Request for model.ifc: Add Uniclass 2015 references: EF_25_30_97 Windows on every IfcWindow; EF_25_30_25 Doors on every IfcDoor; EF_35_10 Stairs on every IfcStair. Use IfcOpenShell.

First a look at what the model holds.

```python
import ifcopenshell

model = ifcopenshell.open("model.ifc")
print(model.schema)
print("classifications:", [c.Name for c in model.by_type("IfcClassification")])
for ifc_class in ("IfcDoor", "IfcRoof", "IfcStair", "IfcWall", "IfcWindow"):
    print(ifc_class, len(model.by_type(ifc_class)))
```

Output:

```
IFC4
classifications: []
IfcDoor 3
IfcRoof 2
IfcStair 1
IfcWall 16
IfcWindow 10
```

```python
import ifcopenshell
import ifcopenshell.api.classification

model = ifcopenshell.open("model.ifc")

system = ifcopenshell.api.classification.add_classification(model, classification="Uniclass 2015")

codes = {
    "IfcWindow": ("EF_25_30_97", "Windows"),
    "IfcDoor": ("EF_25_30_25", "Doors"),
    "IfcStair": ("EF_35_10", "Stairs"),
}
for ifc_class, (code, name) in codes.items():
    products = model.by_type(ifc_class)
    ifcopenshell.api.classification.add_reference(
        model, products=products, classification=system, identification=code, name=name
    )
    print(code, len(products))

model.write("model_v2.ifc")
```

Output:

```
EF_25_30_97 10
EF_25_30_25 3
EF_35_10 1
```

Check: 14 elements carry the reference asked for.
